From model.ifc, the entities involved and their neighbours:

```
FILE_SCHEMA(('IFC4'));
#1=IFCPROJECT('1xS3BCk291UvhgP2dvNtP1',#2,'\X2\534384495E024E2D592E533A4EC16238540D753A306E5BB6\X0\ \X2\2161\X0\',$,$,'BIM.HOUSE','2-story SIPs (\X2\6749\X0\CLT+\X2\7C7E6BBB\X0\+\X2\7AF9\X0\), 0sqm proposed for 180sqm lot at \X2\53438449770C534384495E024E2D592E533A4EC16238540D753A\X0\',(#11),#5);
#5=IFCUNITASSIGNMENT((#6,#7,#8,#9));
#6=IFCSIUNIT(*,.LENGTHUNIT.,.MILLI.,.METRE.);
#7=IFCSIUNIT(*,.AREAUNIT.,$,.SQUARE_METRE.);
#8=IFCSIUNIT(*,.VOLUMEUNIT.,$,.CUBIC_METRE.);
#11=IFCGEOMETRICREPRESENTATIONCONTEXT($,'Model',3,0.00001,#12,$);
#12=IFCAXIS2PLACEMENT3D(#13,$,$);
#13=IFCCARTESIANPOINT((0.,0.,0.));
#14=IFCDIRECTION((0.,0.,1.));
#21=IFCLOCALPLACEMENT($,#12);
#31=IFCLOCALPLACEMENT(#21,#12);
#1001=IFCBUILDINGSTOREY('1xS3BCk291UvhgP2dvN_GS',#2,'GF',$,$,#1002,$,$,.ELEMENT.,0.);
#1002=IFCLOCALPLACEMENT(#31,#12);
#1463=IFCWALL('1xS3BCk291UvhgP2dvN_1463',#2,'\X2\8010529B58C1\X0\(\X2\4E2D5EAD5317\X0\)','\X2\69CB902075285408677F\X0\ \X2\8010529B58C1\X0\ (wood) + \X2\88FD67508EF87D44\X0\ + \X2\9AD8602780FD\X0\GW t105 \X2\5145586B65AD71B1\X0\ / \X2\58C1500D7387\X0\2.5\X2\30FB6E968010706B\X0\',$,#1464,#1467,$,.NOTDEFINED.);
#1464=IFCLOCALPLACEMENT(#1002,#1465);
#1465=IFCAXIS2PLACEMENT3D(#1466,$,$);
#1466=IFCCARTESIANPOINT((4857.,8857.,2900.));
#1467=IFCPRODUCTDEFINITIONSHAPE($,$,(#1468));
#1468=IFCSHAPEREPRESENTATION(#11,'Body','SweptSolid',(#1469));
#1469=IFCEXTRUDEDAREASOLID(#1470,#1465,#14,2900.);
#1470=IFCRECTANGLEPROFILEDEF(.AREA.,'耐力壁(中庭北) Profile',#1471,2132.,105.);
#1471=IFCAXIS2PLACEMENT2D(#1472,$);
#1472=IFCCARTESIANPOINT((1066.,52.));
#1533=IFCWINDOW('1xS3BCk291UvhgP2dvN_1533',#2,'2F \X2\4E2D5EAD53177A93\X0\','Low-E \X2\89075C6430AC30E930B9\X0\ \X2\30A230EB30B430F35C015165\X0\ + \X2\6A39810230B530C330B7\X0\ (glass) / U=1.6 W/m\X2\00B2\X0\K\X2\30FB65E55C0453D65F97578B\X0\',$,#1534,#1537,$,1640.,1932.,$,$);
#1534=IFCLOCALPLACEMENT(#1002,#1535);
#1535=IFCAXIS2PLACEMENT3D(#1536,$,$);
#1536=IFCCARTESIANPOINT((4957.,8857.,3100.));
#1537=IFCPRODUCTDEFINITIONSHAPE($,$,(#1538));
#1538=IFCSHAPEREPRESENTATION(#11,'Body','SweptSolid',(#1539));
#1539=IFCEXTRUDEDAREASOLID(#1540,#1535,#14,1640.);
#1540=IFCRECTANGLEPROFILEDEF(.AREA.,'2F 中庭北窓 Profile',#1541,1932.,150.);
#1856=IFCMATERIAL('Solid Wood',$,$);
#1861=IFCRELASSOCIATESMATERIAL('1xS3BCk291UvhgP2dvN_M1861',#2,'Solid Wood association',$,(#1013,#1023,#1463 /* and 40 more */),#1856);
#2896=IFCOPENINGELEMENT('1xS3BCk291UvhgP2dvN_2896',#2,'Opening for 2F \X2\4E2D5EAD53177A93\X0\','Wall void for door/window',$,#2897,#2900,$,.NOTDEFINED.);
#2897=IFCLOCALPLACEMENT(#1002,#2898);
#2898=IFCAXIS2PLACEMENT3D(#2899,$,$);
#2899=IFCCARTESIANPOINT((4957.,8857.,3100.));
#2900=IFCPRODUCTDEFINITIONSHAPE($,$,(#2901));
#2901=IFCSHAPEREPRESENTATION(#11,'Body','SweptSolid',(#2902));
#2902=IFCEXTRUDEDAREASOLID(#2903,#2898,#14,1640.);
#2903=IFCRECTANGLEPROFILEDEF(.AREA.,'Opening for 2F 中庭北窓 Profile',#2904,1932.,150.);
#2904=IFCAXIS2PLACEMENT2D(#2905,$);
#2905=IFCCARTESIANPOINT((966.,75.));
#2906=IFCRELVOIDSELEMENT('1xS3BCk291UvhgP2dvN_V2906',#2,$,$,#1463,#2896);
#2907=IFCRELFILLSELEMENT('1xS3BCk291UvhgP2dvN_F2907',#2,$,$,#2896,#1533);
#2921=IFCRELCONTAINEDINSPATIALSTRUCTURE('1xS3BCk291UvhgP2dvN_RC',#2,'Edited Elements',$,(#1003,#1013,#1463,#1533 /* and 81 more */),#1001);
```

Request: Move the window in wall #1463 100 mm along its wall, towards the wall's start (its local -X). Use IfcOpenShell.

```python
import ifcopenshell
import ifcopenshell.api.geometry
import ifcopenshell.util.placement

model = ifcopenshell.open("model.ifc")

window = model.by_guid("1xS3BCk291UvhgP2dvN_1533")
opening = window.FillsVoids[0].RelatingOpeningElement
wall = opening.VoidsElements[0].RelatingBuildingElement

wall_matrix = ifcopenshell.util.placement.get_local_placement(wall.ObjectPlacement)
shift = wall_matrix[:3, 0] * -100.0
before = ifcopenshell.util.placement.get_local_placement(window.ObjectPlacement)[:3, 3].copy()

# The window is not placed relative to its opening, so move both.
for product in (opening, window):
    matrix = ifcopenshell.util.placement.get_local_placement(product.ObjectPlacement)
    matrix[:3, 3] += shift
    ifcopenshell.api.geometry.edit_object_placement(model, product=product, matrix=matrix, is_si=False)

after = ifcopenshell.util.placement.get_local_placement(window.ObjectPlacement)[:3, 3]
print("window moved by", (after - before).round(3) + 0.0)

model.write("model_edited.ifc")
```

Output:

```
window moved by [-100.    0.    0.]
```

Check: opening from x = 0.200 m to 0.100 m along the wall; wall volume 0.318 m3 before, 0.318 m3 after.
